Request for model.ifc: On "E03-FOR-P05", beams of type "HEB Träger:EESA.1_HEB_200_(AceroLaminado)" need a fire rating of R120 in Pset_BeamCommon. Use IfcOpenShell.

First a look at what the model holds.

```python
import ifcopenshell
import ifcopenshell.util.element

model = ifcopenshell.open("model.ifc")
print(model.schema)
storey = next(s for s in model.by_type("IfcBuildingStorey") if s.Name == "E03-FOR-P05")
beams = [e for e in ifcopenshell.util.element.get_decomposition(storey) if e.is_a("IfcBeam")]
seen = {}
for e in beams:
    element_type = ifcopenshell.util.element.get_type(e)
    key = (element_type.Name if element_type != e and element_type else None, ifcopenshell.util.element.get_pset(e, "Pset_BeamCommon", "FireRating"))
    seen[key] = seen.get(key, 0) + 1
for (name, value), count in sorted(seen.items(), key=str):
    print(count, "x", name, "|", value)
```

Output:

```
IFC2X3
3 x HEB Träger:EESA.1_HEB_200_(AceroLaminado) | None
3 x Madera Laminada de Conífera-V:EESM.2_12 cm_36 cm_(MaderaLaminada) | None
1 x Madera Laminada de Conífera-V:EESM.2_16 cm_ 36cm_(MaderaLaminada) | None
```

```python
import ifcopenshell
import ifcopenshell.api.pset
import ifcopenshell.util.element

model = ifcopenshell.open("model.ifc")

storey = next(s for s in model.by_type("IfcBuildingStorey") if s.Name == "E03-FOR-P05")
beams = [e for e in ifcopenshell.util.element.get_decomposition(storey) if e.is_a("IfcBeam")]

count = 0
for e in beams:
    element_type = ifcopenshell.util.element.get_type(e)
    if element_type in (None, e) or element_type.Name != "HEB Träger:EESA.1_HEB_200_(AceroLaminado)":
        continue
    # add_pset returns the element's existing set when there is one.
    pset = ifcopenshell.api.pset.add_pset(model, product=e, name="Pset_BeamCommon")
    ifcopenshell.api.pset.edit_pset(model, pset=pset, properties={"FireRating": "R120"})
    count += 1

print(count, "beams updated")

model.write("model_rev.ifc")
```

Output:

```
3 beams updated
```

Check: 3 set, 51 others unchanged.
